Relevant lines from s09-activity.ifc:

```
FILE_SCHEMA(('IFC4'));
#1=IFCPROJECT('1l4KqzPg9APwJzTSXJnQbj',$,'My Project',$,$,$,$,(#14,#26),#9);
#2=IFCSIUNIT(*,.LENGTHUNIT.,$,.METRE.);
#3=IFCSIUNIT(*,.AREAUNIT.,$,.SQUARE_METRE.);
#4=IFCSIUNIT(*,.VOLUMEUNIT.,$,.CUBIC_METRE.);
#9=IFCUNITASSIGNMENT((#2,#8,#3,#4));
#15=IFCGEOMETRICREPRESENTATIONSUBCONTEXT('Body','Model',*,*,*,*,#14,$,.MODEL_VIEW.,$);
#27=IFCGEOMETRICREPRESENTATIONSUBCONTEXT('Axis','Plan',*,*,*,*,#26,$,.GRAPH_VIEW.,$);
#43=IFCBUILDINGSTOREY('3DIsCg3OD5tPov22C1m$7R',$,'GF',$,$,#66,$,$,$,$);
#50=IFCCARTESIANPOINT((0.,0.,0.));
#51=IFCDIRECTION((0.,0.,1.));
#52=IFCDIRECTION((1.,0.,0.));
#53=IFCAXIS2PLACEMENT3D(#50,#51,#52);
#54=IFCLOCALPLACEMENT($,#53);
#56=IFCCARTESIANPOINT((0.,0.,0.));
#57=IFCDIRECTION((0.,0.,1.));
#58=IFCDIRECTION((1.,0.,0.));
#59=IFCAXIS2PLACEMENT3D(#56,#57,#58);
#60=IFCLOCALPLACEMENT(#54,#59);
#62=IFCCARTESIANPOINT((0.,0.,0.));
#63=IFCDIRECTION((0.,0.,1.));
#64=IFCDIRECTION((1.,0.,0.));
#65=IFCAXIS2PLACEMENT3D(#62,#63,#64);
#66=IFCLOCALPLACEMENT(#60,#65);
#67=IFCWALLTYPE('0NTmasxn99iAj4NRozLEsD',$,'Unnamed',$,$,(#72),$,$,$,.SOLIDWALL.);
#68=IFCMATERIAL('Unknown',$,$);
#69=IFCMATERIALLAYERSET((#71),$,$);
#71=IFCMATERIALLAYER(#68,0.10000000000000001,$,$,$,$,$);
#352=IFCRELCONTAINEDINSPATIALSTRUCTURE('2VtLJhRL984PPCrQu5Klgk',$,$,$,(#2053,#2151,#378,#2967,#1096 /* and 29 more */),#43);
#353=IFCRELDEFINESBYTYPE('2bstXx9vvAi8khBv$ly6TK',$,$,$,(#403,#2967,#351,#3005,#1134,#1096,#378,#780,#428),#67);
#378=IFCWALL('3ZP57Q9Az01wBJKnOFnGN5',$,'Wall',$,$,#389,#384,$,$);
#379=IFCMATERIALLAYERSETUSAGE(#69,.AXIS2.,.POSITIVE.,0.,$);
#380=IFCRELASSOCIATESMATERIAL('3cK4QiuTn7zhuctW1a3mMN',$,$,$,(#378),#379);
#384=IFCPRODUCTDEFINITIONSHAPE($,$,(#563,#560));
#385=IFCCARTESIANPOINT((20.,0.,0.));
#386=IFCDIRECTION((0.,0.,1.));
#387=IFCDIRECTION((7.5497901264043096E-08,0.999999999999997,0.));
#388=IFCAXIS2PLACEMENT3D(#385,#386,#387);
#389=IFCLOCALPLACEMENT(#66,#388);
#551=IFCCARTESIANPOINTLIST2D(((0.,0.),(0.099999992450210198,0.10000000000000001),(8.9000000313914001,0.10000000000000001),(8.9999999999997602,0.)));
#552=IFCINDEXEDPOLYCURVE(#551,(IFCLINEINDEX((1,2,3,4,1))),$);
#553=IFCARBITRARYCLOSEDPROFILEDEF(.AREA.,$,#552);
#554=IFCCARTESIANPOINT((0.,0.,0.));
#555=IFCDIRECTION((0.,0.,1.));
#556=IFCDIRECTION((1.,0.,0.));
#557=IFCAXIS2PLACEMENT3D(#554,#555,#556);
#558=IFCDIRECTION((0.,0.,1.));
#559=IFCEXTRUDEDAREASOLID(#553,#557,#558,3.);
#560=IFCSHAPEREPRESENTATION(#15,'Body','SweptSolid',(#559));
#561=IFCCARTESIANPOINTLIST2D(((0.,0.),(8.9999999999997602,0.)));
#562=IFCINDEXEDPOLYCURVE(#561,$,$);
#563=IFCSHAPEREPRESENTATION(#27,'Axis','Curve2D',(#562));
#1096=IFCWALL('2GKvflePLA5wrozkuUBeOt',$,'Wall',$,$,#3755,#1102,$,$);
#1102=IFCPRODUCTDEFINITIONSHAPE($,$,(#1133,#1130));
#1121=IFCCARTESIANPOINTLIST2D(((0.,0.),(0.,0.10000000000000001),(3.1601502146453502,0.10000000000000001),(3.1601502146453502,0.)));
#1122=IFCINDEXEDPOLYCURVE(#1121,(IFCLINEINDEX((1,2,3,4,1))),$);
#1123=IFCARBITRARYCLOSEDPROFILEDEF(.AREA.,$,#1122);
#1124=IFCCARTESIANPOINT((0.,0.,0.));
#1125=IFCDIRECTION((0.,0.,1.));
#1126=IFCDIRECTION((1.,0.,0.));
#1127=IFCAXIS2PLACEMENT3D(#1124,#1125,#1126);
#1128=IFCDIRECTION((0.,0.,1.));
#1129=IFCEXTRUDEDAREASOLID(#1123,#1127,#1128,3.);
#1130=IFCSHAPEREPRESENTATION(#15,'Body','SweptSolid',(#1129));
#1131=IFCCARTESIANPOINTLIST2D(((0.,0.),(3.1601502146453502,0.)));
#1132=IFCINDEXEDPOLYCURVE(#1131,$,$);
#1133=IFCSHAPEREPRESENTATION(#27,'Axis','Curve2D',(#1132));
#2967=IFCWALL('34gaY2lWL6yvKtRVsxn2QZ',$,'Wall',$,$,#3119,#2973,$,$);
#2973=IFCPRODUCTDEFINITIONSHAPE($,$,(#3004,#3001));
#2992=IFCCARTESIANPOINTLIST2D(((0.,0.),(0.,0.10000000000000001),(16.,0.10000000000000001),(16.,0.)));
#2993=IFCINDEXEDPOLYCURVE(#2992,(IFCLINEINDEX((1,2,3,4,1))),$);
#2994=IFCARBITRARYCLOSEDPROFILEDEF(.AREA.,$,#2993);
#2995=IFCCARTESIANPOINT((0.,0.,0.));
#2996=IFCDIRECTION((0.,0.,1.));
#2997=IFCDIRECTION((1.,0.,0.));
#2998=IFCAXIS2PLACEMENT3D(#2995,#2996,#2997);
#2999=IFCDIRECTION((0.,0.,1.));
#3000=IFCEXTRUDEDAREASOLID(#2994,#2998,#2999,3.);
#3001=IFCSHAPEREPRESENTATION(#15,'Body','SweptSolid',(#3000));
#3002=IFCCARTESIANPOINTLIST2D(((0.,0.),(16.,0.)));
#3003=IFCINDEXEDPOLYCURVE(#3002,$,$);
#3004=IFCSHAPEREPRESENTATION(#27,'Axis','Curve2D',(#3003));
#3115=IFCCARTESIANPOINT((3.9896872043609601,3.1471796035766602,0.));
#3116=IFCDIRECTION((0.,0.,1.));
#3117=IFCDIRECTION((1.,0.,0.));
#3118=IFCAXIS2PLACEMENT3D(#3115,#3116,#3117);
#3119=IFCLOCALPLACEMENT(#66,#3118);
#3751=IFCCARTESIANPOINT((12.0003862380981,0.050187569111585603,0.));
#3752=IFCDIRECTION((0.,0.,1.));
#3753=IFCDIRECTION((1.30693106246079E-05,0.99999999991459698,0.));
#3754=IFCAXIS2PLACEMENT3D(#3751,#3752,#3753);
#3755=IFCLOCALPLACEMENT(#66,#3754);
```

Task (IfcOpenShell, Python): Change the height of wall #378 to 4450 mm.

```python
import ifcopenshell
import ifcopenshell.geom
import ifcopenshell.util.representation
import ifcopenshell.util.shape

model = ifcopenshell.open("s09-activity.ifc")
settings = ifcopenshell.geom.settings()


def volume(element):
    """Net volume in cubic metres, openings subtracted."""
    shape = ifcopenshell.geom.create_shape(settings, element)
    return ifcopenshell.util.shape.get_volume(shape.geometry)


wall = model.by_id(378)
before = volume(wall)

body = ifcopenshell.util.representation.get_representation(wall, "Model", "Body")
solid = body.Items[0]
old_height = solid.Depth
solid.Depth = 4.45
after = volume(wall)

print(f"height {old_height:g} -> {solid.Depth:g}, volume {before:.3f} -> {after:.3f} m3")

model.write("s09-activity-out.ifc")
```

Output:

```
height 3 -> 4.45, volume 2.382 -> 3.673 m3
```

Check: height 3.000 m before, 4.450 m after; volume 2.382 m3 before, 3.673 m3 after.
